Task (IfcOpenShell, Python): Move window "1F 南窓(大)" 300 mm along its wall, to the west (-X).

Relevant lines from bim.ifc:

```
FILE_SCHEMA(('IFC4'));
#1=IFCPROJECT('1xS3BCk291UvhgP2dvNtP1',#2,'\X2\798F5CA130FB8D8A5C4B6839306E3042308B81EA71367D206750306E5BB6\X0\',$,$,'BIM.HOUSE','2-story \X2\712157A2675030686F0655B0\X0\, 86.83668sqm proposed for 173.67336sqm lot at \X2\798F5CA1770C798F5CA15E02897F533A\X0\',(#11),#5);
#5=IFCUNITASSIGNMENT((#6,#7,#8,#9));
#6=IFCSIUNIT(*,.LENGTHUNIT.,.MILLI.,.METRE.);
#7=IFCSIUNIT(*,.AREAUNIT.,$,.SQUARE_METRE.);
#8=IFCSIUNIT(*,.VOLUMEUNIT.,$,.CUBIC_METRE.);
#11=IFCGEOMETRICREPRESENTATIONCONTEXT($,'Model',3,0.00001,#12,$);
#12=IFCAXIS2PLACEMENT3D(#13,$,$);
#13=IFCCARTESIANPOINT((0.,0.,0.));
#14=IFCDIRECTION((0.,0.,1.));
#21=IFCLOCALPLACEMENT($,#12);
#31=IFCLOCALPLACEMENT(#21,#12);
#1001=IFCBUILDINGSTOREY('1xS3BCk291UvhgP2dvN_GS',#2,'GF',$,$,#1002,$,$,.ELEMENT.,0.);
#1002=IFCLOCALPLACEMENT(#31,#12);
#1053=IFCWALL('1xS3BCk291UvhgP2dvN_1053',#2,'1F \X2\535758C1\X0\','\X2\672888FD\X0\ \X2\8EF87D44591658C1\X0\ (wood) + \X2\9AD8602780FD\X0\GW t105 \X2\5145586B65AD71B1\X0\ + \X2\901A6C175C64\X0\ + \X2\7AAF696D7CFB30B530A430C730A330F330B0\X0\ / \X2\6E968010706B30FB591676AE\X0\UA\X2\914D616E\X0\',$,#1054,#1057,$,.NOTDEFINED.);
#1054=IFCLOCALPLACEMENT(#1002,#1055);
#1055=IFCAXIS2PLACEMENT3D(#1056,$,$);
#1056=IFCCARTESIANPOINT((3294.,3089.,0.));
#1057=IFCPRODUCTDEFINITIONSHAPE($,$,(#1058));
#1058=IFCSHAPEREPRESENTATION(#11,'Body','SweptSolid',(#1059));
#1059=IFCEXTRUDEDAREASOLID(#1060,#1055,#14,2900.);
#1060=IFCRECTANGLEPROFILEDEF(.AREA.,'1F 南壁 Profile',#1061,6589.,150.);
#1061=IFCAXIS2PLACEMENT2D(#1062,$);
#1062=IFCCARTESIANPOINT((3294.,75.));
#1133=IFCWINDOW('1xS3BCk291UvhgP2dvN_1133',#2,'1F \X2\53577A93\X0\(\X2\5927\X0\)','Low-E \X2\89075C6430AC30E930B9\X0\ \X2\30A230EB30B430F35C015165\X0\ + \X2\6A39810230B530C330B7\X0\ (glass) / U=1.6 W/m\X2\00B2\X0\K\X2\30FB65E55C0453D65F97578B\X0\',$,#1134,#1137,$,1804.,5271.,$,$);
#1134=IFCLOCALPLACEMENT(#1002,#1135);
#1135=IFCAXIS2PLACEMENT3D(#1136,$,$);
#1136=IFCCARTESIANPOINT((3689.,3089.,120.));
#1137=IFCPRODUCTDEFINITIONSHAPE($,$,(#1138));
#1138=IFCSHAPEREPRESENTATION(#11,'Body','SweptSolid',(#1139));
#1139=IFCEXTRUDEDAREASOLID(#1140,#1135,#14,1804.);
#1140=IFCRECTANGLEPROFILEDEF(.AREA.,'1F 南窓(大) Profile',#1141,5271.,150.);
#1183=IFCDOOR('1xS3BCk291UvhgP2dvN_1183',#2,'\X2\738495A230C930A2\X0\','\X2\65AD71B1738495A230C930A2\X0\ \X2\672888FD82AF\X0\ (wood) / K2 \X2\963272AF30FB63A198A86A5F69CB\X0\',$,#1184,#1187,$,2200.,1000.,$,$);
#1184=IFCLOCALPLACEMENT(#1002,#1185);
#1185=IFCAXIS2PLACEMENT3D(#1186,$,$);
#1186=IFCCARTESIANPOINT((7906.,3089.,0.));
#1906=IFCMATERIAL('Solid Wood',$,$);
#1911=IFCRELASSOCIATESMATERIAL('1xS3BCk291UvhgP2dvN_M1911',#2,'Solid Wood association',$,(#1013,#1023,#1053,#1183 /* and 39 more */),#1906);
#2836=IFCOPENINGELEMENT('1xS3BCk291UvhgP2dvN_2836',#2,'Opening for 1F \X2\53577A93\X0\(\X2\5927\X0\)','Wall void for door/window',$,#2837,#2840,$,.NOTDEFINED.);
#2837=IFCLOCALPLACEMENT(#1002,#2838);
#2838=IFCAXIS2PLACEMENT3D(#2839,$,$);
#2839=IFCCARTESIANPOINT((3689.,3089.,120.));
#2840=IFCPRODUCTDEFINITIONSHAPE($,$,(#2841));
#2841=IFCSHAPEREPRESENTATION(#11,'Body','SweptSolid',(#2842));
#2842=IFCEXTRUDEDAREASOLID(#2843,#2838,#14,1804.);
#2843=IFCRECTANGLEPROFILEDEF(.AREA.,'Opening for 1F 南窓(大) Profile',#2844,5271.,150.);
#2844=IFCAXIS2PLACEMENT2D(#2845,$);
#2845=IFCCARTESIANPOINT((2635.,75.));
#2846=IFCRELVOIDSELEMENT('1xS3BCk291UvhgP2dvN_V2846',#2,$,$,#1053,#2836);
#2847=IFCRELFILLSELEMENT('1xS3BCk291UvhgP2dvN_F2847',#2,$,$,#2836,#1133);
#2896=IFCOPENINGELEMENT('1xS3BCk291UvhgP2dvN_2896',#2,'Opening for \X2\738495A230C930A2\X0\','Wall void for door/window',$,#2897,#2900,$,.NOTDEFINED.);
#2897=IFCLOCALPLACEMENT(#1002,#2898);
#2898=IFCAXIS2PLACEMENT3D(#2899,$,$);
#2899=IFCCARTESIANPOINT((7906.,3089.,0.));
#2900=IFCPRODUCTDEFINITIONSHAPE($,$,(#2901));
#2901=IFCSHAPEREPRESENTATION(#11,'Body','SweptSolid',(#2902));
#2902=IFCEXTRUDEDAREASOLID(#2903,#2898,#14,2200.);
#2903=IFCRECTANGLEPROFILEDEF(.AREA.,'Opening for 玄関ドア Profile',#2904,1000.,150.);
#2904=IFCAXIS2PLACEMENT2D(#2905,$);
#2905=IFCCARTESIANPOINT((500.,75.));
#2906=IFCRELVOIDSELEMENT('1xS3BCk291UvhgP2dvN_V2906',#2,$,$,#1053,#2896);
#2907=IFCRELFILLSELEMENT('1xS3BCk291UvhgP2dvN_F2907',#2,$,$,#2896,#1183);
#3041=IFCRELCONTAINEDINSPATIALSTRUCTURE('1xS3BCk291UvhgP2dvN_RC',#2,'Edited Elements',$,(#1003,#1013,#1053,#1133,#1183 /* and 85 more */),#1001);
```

```python
import ifcopenshell
import ifcopenshell.api.geometry
import ifcopenshell.util.placement

model = ifcopenshell.open("bim.ifc")

window = model.by_id(1133)
opening = window.FillsVoids[0].RelatingOpeningElement
wall = opening.VoidsElements[0].RelatingBuildingElement

wall_matrix = ifcopenshell.util.placement.get_local_placement(wall.ObjectPlacement)
shift = wall_matrix[:3, 0] * -300.0
before = ifcopenshell.util.placement.get_local_placement(window.ObjectPlacement)[:3, 3].copy()

# The window is not placed relative to its opening, so move both.
for product in (opening, window):
    matrix = ifcopenshell.util.placement.get_local_placement(product.ObjectPlacement)
    matrix[:3, 3] += shift
    ifcopenshell.api.geometry.edit_object_placement(model, product=product, matrix=matrix, is_si=False)

after = ifcopenshell.util.placement.get_local_placement(window.ObjectPlacement)[:3, 3]
print("window moved by", (after - before).round(3) + 0.0)

model.write("bim_rev.ifc")
```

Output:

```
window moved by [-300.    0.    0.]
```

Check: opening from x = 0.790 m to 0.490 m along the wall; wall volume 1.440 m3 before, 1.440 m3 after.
